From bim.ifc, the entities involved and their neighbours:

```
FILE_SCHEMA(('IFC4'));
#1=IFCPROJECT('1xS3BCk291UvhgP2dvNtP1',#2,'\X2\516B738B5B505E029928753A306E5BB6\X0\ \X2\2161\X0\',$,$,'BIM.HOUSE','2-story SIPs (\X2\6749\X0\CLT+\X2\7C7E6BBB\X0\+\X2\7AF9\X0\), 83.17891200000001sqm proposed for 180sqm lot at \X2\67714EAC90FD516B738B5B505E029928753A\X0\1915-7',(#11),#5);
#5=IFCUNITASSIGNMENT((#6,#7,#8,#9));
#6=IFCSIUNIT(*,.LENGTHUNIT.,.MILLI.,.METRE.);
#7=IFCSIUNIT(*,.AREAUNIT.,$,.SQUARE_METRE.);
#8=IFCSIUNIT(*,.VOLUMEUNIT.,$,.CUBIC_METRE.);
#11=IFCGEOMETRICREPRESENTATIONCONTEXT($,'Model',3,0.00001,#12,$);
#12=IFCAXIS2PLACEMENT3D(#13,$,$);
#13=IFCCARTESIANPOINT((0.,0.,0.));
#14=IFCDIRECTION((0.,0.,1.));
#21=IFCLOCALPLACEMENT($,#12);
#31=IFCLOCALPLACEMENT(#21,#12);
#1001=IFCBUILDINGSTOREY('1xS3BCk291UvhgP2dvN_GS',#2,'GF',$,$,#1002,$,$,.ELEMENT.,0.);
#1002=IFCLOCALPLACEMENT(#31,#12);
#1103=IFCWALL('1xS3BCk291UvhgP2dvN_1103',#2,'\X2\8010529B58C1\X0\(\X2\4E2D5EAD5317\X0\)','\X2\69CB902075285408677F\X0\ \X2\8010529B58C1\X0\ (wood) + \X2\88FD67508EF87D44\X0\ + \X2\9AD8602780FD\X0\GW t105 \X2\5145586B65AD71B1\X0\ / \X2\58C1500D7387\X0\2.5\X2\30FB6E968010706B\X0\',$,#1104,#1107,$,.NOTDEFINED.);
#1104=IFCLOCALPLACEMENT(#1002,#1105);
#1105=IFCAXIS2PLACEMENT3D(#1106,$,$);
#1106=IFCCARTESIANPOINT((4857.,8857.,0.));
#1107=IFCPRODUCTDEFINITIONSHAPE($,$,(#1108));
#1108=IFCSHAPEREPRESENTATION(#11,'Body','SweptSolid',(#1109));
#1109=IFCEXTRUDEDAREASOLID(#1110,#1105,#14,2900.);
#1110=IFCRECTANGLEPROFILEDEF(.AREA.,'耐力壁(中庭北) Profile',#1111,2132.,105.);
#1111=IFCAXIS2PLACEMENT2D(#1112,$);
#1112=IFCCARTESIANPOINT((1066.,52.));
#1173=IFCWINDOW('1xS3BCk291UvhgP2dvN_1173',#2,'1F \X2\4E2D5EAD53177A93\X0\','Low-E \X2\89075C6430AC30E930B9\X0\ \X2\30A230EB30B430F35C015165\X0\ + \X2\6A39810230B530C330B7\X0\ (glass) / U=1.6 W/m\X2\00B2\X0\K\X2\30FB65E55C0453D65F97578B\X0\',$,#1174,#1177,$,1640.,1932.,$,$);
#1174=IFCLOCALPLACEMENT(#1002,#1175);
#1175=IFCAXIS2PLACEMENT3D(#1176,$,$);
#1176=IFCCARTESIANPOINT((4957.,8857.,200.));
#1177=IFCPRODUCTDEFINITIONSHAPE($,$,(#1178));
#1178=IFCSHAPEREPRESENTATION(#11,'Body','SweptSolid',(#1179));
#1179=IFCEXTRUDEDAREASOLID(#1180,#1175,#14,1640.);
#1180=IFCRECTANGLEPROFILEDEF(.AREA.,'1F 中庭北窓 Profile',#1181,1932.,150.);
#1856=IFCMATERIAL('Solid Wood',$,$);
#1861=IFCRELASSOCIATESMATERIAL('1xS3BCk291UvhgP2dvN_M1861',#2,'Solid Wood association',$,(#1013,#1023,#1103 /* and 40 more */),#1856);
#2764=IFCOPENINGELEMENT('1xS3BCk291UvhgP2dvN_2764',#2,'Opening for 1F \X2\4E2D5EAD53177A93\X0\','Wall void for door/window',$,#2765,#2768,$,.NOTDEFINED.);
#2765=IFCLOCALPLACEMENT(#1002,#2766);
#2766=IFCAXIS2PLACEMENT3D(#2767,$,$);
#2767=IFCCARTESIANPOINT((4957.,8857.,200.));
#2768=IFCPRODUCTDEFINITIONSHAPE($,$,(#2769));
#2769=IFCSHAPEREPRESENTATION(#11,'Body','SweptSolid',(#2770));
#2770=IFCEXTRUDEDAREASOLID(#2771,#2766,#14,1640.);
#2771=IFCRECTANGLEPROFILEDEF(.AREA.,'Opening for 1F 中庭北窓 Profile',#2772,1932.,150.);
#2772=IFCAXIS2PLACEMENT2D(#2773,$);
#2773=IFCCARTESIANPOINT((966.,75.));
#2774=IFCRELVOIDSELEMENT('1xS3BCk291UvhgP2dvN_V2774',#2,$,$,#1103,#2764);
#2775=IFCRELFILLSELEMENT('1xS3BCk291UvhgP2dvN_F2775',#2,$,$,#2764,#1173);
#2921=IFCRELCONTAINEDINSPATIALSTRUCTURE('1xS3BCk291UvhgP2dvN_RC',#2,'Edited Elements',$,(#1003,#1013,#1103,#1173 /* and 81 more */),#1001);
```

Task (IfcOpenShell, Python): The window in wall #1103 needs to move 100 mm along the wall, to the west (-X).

```python
import ifcopenshell
import ifcopenshell.api.geometry
import ifcopenshell.util.placement

model = ifcopenshell.open("bim.ifc")

window = model.by_guid("1xS3BCk291UvhgP2dvN_1173")
opening = window.FillsVoids[0].RelatingOpeningElement
wall = opening.VoidsElements[0].RelatingBuildingElement

wall_matrix = ifcopenshell.util.placement.get_local_placement(wall.ObjectPlacement)
shift = wall_matrix[:3, 0] * -100.0
before = ifcopenshell.util.placement.get_local_placement(window.ObjectPlacement)[:3, 3].copy()

# The window is not placed relative to its opening, so move both.
for product in (opening, window):
    matrix = ifcopenshell.util.placement.get_local_placement(product.ObjectPlacement)
    matrix[:3, 3] += shift
    ifcopenshell.api.geometry.edit_object_placement(model, product=product, matrix=matrix, is_si=False)

after = ifcopenshell.util.placement.get_local_placement(window.ObjectPlacement)[:3, 3]
print("window moved by", (after - before).round(3) + 0.0)

model.write("bim_updated.ifc")
```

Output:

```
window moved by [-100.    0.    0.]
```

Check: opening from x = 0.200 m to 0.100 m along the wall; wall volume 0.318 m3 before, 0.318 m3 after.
